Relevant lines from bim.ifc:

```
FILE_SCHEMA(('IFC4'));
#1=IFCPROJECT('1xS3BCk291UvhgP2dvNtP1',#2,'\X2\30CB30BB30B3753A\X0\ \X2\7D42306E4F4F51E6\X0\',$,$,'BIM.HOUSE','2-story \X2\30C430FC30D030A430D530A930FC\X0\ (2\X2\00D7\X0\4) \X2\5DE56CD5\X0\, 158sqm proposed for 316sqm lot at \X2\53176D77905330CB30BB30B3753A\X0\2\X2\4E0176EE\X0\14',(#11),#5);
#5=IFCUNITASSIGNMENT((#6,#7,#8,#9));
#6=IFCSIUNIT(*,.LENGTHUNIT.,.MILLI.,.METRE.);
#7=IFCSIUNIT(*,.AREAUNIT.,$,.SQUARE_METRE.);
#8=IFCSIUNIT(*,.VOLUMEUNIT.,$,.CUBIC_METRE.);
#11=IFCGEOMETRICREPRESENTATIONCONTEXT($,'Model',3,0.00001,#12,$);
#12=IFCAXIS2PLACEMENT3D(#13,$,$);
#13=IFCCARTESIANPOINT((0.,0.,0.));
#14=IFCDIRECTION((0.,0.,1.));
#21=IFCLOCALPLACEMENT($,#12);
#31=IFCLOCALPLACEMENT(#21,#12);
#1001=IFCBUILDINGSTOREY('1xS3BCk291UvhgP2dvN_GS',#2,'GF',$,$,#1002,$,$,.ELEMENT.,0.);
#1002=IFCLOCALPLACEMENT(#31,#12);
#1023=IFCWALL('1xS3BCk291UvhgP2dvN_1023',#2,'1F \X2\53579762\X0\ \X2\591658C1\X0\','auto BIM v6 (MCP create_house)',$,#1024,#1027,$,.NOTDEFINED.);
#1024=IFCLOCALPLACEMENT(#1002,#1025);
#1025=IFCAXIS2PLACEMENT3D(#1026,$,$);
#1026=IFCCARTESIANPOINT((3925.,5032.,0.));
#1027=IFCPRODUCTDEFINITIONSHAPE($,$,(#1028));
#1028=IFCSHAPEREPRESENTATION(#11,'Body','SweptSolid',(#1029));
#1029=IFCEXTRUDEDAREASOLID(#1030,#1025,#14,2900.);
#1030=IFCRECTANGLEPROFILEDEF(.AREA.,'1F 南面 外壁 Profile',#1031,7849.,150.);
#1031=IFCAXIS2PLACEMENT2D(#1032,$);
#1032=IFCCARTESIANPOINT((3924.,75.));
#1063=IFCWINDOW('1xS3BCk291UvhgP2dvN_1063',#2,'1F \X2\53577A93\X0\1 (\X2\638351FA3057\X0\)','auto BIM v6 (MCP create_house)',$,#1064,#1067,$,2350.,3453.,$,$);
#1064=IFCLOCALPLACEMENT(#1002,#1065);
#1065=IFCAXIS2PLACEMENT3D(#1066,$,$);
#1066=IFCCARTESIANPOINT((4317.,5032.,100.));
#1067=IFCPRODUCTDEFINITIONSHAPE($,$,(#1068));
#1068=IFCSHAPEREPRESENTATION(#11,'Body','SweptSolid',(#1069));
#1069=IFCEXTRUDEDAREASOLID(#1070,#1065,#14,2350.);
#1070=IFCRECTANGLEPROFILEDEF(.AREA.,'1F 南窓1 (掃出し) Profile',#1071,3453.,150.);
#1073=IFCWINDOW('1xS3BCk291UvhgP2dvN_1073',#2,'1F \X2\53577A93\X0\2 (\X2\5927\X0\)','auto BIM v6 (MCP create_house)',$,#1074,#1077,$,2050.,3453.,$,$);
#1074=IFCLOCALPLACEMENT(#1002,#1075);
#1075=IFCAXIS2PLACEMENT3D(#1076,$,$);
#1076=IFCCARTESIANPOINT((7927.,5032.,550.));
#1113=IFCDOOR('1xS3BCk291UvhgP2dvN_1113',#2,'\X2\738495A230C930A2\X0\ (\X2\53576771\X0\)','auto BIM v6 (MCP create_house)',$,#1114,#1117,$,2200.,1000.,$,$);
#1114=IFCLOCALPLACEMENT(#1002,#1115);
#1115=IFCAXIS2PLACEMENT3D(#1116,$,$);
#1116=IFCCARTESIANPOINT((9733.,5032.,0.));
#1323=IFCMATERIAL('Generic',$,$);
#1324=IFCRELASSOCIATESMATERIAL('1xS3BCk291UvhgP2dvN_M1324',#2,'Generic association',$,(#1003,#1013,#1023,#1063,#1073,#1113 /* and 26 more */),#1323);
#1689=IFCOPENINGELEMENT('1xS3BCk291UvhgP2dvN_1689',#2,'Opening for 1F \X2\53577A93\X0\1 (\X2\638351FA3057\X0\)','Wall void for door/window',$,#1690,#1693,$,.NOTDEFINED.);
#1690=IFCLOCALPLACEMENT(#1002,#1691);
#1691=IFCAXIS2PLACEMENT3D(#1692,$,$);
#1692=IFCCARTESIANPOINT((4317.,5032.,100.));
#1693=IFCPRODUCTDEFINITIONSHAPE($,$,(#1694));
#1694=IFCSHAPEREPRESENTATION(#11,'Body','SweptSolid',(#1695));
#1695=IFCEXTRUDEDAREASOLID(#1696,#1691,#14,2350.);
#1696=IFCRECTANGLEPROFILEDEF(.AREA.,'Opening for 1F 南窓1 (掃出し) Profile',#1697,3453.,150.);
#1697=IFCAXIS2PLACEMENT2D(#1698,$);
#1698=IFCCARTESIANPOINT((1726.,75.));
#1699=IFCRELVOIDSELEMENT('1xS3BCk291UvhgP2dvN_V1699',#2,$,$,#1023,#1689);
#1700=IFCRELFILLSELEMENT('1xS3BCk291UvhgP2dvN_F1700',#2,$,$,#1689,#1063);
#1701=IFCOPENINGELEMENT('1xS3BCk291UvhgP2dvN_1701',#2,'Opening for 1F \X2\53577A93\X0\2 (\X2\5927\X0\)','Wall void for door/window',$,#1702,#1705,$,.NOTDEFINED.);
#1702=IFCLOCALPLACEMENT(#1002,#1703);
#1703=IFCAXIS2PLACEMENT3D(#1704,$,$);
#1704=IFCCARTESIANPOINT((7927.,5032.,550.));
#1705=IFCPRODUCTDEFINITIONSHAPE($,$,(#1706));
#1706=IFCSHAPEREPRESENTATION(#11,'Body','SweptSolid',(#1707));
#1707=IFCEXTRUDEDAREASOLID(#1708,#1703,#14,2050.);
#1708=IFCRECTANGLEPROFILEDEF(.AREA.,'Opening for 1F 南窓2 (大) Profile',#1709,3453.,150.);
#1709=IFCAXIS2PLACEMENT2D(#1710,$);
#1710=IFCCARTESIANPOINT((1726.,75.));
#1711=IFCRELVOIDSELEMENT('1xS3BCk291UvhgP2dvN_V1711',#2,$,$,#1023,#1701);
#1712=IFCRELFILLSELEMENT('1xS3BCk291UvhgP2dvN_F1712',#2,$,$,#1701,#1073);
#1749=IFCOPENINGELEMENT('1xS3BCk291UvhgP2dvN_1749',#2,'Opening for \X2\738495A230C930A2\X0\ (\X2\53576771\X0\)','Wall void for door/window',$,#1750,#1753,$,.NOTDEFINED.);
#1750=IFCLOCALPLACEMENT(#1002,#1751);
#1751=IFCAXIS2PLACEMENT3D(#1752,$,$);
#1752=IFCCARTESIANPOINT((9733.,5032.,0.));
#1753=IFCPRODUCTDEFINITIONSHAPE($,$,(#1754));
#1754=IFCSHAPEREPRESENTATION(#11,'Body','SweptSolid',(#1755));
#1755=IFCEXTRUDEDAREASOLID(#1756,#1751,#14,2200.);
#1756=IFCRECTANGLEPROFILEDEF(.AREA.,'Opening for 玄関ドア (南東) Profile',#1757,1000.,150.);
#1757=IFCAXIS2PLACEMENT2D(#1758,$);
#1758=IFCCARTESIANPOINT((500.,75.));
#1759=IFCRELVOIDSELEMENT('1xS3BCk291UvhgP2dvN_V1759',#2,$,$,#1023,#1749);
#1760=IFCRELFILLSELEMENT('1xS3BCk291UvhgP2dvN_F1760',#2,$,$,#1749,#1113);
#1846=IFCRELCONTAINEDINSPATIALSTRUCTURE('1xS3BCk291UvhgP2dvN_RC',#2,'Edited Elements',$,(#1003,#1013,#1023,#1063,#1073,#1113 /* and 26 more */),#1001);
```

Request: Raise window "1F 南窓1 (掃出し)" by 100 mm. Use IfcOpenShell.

```python
import numpy as np
import ifcopenshell
import ifcopenshell.api.geometry
import ifcopenshell.util.placement
import ifcopenshell.util.unit

model = ifcopenshell.open("bim.ifc")
unit_scale = ifcopenshell.util.unit.calculate_unit_scale(model)

window = model.by_guid("1xS3BCk291UvhgP2dvN_1063")
opening = window.FillsVoids[0].RelatingOpeningElement
dz = 0.1 / unit_scale

shift = np.array([0.0, 0.0, dz])
# The window is not placed relative to its opening, so move both.
for product in (opening, window):
    matrix = ifcopenshell.util.placement.get_local_placement(product.ObjectPlacement)
    matrix[:3, 3] += shift
    ifcopenshell.api.geometry.edit_object_placement(model, product=product, matrix=matrix, is_si=False)

print(f"moved by {dz * unit_scale:+.3f} m")

model.write("bim_updated.ifc")
```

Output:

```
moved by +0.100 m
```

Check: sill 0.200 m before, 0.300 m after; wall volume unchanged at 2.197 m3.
